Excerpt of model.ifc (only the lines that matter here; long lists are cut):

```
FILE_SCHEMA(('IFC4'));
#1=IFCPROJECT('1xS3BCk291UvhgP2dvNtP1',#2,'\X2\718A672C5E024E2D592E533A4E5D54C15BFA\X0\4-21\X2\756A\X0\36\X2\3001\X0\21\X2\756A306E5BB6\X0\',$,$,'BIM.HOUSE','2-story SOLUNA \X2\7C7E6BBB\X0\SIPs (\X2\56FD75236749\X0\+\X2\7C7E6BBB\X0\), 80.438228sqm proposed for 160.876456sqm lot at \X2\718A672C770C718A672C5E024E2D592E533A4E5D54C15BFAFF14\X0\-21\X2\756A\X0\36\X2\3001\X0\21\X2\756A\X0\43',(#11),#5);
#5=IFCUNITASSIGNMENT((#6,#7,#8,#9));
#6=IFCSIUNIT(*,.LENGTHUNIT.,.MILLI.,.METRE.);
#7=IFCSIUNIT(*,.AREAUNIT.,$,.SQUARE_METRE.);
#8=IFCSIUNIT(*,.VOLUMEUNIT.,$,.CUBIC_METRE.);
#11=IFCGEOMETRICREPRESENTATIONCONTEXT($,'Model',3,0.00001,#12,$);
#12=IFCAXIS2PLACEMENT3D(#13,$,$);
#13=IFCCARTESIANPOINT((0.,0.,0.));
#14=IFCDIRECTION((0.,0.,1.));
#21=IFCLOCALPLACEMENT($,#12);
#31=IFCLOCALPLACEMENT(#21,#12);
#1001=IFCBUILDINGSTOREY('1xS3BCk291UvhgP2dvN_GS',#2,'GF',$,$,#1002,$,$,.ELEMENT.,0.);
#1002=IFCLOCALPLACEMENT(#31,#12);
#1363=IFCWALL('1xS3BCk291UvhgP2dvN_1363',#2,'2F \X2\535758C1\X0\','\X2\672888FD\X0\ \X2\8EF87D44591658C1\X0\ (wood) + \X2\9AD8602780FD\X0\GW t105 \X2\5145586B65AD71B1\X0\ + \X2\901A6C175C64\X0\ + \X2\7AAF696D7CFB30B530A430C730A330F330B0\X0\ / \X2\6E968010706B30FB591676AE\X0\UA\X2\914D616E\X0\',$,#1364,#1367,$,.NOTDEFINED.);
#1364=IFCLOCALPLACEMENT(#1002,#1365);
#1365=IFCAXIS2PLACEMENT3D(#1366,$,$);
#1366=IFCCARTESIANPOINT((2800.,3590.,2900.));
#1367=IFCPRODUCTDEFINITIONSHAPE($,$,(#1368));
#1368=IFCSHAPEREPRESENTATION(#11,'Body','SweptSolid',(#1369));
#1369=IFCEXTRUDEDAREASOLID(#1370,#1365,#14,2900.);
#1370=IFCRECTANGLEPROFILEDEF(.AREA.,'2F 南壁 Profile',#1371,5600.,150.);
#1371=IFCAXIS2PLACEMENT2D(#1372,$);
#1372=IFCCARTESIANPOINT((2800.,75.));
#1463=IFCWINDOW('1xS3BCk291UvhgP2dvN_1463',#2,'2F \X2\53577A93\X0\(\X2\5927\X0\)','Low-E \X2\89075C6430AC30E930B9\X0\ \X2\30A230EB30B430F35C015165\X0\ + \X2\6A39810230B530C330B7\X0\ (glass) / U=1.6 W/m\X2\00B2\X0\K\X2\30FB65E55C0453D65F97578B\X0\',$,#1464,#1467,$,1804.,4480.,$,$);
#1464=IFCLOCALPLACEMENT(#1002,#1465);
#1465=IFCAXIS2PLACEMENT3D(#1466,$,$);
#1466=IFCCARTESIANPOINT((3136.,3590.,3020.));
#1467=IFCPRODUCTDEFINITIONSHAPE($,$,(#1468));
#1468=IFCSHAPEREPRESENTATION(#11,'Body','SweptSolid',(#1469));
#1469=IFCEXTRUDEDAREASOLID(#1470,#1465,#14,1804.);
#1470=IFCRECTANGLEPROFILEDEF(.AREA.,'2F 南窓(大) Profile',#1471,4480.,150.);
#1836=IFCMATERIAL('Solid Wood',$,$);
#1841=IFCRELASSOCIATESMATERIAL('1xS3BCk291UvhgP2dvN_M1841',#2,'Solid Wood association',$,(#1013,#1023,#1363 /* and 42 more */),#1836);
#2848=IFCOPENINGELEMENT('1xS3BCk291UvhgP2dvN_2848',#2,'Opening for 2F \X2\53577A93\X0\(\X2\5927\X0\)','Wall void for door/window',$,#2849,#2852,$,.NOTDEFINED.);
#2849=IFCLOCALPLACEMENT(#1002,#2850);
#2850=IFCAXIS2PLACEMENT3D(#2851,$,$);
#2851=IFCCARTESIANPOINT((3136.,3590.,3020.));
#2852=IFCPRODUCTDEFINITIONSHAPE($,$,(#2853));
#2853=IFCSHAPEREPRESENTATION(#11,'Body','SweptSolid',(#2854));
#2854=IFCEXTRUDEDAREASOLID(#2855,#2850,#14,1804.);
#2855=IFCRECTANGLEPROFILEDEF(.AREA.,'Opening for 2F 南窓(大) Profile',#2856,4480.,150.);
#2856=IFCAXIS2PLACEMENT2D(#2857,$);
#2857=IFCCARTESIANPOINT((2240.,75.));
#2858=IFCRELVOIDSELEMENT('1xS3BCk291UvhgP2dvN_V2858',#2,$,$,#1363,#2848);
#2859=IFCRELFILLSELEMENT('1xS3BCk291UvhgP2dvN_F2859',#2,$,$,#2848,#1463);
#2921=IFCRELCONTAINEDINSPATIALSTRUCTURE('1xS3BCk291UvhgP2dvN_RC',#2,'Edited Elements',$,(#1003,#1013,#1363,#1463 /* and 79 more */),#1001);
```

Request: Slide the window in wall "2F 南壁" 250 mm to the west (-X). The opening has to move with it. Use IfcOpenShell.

```python
import ifcopenshell
import ifcopenshell.api.geometry
import ifcopenshell.util.placement
import ifcopenshell.util.unit

model = ifcopenshell.open("model.ifc")
unit_scale = ifcopenshell.util.unit.calculate_unit_scale(model)

window = model.by_guid("1xS3BCk291UvhgP2dvN_1463")
opening = window.FillsVoids[0].RelatingOpeningElement
wall = opening.VoidsElements[0].RelatingBuildingElement

wall_matrix = ifcopenshell.util.placement.get_local_placement(wall.ObjectPlacement)
shift = wall_matrix[:3, 0] * -0.25 / unit_scale
before = ifcopenshell.util.placement.get_local_placement(window.ObjectPlacement)[:3, 3].copy()

# The window is not placed relative to its opening, so move both.
for product in (opening, window):
    matrix = ifcopenshell.util.placement.get_local_placement(product.ObjectPlacement)
    matrix[:3, 3] += shift
    ifcopenshell.api.geometry.edit_object_placement(model, product=product, matrix=matrix, is_si=False)

after = ifcopenshell.util.placement.get_local_placement(window.ObjectPlacement)[:3, 3]
print("window moved by", (after - before).round(3) + 0.0)

model.write("model_v2.ifc")
```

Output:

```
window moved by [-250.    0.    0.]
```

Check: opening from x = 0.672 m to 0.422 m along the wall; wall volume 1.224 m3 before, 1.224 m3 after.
